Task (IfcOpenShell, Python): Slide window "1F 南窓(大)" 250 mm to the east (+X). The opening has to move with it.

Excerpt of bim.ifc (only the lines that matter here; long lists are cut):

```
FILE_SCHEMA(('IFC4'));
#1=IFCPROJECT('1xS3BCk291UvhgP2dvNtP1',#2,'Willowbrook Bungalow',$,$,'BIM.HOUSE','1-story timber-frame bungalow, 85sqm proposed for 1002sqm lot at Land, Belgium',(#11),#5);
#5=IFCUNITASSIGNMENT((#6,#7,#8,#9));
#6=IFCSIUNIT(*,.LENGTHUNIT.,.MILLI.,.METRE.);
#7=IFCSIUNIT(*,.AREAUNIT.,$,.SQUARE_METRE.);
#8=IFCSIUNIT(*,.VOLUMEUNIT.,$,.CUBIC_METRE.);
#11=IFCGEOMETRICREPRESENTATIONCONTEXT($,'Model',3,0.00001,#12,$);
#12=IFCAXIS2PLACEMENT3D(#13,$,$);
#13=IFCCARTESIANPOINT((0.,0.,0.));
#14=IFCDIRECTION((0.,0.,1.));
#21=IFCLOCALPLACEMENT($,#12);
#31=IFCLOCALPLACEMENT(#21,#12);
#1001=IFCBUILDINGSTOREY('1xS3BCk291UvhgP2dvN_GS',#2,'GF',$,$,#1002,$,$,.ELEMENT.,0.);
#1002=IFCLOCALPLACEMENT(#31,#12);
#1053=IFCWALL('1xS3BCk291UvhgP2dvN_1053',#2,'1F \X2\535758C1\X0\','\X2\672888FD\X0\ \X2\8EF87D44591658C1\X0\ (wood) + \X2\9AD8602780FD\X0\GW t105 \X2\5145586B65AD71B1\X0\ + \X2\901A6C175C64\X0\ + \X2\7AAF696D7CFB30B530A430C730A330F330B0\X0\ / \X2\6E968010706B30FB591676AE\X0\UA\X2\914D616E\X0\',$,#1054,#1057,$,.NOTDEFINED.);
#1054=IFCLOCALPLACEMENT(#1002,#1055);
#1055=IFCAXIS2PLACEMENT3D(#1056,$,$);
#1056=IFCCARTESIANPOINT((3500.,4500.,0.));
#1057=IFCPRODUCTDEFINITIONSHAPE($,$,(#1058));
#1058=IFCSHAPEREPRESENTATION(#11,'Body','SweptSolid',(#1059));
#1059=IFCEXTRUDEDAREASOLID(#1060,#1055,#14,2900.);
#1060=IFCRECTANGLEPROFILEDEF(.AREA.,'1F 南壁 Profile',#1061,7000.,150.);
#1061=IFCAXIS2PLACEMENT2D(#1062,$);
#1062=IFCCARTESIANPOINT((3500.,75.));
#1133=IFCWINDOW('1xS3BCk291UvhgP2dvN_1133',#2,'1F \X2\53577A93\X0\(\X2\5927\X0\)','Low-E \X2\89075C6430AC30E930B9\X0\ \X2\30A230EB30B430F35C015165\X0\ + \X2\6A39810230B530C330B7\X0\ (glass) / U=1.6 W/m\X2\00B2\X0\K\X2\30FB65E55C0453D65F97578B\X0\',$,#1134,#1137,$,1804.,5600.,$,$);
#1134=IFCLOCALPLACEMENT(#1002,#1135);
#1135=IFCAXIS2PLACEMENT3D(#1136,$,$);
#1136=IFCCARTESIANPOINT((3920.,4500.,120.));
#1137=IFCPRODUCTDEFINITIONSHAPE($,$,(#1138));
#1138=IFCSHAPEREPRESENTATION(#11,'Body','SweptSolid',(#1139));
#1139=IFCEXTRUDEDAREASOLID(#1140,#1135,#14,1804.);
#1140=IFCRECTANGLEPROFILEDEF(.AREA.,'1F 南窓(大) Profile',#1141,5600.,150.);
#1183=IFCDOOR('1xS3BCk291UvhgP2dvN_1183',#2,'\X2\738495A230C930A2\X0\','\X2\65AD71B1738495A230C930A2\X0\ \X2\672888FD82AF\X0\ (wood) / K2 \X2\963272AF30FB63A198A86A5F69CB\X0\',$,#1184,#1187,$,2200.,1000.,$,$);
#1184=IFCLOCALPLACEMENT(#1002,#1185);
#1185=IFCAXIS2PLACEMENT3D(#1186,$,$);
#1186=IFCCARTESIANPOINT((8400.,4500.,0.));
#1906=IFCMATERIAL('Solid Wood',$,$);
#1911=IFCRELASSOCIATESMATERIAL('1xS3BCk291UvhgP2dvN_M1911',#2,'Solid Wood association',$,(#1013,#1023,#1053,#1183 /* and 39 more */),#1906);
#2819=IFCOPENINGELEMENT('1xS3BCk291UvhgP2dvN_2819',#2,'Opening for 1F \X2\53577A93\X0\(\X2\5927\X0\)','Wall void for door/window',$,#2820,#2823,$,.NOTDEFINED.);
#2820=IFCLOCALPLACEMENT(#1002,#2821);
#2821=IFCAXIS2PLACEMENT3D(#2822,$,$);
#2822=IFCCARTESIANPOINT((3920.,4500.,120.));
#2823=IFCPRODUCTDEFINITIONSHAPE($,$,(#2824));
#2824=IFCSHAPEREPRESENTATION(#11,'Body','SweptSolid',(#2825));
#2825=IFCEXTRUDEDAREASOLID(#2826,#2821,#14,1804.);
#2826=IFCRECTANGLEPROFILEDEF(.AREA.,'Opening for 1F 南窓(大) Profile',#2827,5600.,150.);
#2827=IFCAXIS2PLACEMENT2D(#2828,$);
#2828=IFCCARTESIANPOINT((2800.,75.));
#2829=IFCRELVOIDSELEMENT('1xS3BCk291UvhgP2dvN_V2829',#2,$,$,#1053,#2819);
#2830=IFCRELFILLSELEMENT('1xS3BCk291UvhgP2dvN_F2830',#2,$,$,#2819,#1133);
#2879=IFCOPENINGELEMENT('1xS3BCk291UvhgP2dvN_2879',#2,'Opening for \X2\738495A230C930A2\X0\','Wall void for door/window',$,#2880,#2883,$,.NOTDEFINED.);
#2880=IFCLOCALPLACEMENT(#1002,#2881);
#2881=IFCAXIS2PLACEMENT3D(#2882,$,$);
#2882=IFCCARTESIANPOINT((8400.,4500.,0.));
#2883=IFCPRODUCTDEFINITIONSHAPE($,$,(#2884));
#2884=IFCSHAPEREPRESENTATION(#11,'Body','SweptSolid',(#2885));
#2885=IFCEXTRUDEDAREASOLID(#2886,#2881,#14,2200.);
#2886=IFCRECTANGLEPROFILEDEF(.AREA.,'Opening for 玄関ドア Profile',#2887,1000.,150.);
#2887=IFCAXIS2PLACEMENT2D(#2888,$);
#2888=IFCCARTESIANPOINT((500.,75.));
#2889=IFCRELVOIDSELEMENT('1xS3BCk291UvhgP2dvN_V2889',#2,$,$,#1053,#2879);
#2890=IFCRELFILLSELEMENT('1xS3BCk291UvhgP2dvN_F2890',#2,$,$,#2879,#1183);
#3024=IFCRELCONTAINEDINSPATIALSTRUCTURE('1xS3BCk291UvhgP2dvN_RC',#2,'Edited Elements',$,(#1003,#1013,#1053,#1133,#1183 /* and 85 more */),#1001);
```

```python
import ifcopenshell
import ifcopenshell.api.geometry
import ifcopenshell.util.placement
import ifcopenshell.util.unit

model = ifcopenshell.open("bim.ifc")
unit_scale = ifcopenshell.util.unit.calculate_unit_scale(model)

window = model.by_id(1133)
opening = window.FillsVoids[0].RelatingOpeningElement
wall = opening.VoidsElements[0].RelatingBuildingElement

wall_matrix = ifcopenshell.util.placement.get_local_placement(wall.ObjectPlacement)
shift = wall_matrix[:3, 0] * 0.25 / unit_scale
before = ifcopenshell.util.placement.get_local_placement(window.ObjectPlacement)[:3, 3].copy()

# The window is not placed relative to its opening, so move both.
for product in (opening, window):
    matrix = ifcopenshell.util.placement.get_local_placement(product.ObjectPlacement)
    matrix[:3, 3] += shift
    ifcopenshell.api.geometry.edit_object_placement(model, product=product, matrix=matrix, is_si=False)

after = ifcopenshell.util.placement.get_local_placement(window.ObjectPlacement)[:3, 3]
print("window moved by", (after - before).round(3) + 0.0)

model.write("bim_edited.ifc")
```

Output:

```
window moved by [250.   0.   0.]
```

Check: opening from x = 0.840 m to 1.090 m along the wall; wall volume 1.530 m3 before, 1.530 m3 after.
